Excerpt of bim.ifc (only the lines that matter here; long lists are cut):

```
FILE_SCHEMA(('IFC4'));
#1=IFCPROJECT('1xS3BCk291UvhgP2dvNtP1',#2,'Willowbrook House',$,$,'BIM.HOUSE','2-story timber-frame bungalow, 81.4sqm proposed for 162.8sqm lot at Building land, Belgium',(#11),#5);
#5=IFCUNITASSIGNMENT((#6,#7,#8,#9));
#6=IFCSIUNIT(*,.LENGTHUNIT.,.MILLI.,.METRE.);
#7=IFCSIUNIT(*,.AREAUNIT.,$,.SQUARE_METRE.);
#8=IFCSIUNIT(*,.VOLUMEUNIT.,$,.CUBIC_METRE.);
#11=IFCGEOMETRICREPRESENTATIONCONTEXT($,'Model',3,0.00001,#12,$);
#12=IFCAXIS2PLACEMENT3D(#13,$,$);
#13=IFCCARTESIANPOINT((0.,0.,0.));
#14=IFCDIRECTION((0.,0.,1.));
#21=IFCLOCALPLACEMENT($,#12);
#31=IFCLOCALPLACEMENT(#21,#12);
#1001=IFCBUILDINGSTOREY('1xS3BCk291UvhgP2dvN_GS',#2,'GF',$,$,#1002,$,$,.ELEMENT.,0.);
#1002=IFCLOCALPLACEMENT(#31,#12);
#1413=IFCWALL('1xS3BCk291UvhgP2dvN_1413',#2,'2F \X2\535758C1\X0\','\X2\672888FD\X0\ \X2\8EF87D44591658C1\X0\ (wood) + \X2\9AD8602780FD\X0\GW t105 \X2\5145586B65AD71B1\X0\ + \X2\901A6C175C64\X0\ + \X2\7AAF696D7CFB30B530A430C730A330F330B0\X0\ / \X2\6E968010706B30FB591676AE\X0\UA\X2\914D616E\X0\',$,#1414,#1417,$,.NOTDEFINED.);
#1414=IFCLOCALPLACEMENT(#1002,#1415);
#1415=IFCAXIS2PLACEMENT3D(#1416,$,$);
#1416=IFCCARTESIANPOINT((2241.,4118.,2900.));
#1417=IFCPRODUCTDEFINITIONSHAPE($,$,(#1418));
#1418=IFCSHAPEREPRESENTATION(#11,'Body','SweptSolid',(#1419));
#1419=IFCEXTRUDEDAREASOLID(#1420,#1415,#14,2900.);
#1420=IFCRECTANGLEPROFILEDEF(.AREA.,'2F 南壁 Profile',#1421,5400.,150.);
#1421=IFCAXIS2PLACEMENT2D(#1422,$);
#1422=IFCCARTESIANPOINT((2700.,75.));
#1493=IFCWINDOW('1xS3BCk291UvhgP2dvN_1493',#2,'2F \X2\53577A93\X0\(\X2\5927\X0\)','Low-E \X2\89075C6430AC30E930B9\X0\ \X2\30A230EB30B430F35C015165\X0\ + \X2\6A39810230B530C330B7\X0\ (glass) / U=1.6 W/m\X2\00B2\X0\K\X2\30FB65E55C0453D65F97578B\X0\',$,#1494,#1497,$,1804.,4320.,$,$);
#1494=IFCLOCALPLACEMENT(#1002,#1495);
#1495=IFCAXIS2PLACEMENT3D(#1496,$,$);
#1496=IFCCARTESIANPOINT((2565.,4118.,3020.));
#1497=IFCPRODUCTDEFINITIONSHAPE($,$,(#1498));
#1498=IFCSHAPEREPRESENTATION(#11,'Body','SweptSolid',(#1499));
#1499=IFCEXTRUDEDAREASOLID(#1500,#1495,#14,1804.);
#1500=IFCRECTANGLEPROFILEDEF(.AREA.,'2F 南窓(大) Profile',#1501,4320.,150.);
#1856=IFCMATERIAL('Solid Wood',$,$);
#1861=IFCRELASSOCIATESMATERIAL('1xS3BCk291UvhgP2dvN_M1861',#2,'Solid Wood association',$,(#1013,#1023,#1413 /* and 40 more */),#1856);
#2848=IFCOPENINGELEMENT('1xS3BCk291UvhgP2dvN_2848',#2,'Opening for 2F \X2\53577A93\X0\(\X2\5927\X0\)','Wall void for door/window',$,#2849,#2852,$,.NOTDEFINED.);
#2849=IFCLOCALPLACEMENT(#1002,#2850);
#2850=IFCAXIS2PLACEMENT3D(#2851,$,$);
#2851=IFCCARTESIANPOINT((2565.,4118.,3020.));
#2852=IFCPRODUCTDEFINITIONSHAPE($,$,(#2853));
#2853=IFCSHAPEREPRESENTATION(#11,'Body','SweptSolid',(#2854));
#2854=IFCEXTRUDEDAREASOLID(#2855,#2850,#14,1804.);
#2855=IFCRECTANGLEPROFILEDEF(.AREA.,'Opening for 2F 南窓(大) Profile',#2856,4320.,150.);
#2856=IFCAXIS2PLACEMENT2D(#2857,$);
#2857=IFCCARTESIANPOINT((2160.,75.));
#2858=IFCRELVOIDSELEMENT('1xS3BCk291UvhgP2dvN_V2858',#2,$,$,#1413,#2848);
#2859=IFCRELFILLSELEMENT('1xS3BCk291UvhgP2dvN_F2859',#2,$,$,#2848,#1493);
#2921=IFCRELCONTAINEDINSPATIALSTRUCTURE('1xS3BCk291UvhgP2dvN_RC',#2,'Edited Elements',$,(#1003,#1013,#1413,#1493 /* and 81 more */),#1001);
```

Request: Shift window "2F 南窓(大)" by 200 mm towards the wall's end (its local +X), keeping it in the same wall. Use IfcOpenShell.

```python
import ifcopenshell
import ifcopenshell.api.geometry
import ifcopenshell.util.placement
import ifcopenshell.util.unit

model = ifcopenshell.open("bim.ifc")
unit_scale = ifcopenshell.util.unit.calculate_unit_scale(model)

window = model.by_id(1493)
opening = window.FillsVoids[0].RelatingOpeningElement
wall = opening.VoidsElements[0].RelatingBuildingElement

wall_matrix = ifcopenshell.util.placement.get_local_placement(wall.ObjectPlacement)
shift = wall_matrix[:3, 0] * 0.2 / unit_scale
before = ifcopenshell.util.placement.get_local_placement(window.ObjectPlacement)[:3, 3].copy()

# The window is not placed relative to its opening, so move both.
for product in (opening, window):
    matrix = ifcopenshell.util.placement.get_local_placement(product.ObjectPlacement)
    matrix[:3, 3] += shift
    ifcopenshell.api.geometry.edit_object_placement(model, product=product, matrix=matrix, is_si=False)

after = ifcopenshell.util.placement.get_local_placement(window.ObjectPlacement)[:3, 3]
print("window moved by", (after - before).round(3) + 0.0)

model.write("bim_updated.ifc")
```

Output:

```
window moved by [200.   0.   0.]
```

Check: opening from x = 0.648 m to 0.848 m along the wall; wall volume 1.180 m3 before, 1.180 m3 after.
